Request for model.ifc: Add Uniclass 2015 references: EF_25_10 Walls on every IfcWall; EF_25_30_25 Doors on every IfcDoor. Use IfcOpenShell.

First a look at what the model holds.

```python
import ifcopenshell

model = ifcopenshell.open("model.ifc")
print(model.schema)
print("classifications:", [c.Name for c in model.by_type("IfcClassification")])
for ifc_class in ("IfcDoor", "IfcRoof", "IfcStair", "IfcWall", "IfcWindow"):
    print(ifc_class, len(model.by_type(ifc_class)))
```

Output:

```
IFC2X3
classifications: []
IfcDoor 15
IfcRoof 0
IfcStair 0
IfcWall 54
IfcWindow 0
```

```python
import ifcopenshell
import ifcopenshell.api.classification

model = ifcopenshell.open("model.ifc")

# IFC2X3 requires Source and Edition and has no link from the project to the system.
system = model.create_entity("IfcClassification", Source="NBS", Edition="2015", Name="Uniclass 2015")

codes = {
    "IfcWall": ("EF_25_10", "Walls"),
    "IfcDoor": ("EF_25_30_25", "Doors"),
}
for ifc_class, (code, name) in codes.items():
    products = model.by_type(ifc_class)
    ifcopenshell.api.classification.add_reference(
        model, products=products, classification=system, identification=code, name=name
    )
    print(code, len(products))

model.write("model_edited.ifc")
```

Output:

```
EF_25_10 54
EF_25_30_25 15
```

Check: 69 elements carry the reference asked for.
